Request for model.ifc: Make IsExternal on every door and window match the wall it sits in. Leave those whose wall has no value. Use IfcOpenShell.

First a look at what the model holds.

```python
import ifcopenshell
import ifcopenshell.util.element

model = ifcopenshell.open("model.ifc")
print(model.schema)
seen = {}
for e in model.by_type("IfcDoor") + model.by_type("IfcWindow"):
    if not e.FillsVoids:
        continue
    host = e.FillsVoids[0].RelatingOpeningElement.VoidsElements[0].RelatingBuildingElement
    own = ifcopenshell.util.element.get_pset(e, f"Pset_{e.is_a()[3:].removesuffix('StandardCase')}Common", "IsExternal")
    wall = ifcopenshell.util.element.get_pset(host, "Pset_WallCommon", "IsExternal")
    seen[e.is_a(), own, wall] = seen.get((e.is_a(), own, wall), 0) + 1
for (cls, own, wall), count in sorted(seen.items(), key=str):
    print(count, cls, "IsExternal:", own, "| host wall:", wall)
```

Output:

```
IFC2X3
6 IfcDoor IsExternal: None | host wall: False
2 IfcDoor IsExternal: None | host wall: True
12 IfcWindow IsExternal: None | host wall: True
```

```python
import ifcopenshell
import ifcopenshell.api.pset
import ifcopenshell.util.element

model = ifcopenshell.open("model.ifc")

count = 0
for ifc_class, pset_name in (("IfcDoor", "Pset_DoorCommon"), ("IfcWindow", "Pset_WindowCommon")):
    for e in model.by_type(ifc_class):
        if not e.FillsVoids:
            continue
        host = e.FillsVoids[0].RelatingOpeningElement.VoidsElements[0].RelatingBuildingElement
        external = ifcopenshell.util.element.get_pset(host, "Pset_WallCommon", "IsExternal")
        if external is None or ifcopenshell.util.element.get_pset(e, pset_name, "IsExternal") == external:
            continue
        pset = ifcopenshell.api.pset.add_pset(model, product=e, name=pset_name)
        ifcopenshell.api.pset.edit_pset(model, pset=pset, properties={"IsExternal": external})
        count += 1

print(count, "updated")

model.write("model_rev.ifc")
```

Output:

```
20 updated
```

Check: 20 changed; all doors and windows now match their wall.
